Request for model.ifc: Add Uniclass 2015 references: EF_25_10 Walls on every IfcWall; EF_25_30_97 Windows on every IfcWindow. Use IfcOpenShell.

First a look at what the model holds.

```python
import ifcopenshell

model = ifcopenshell.open("model.ifc")
print(model.schema)
print("classifications:", [c.Name for c in model.by_type("IfcClassification")])
for ifc_class in ("IfcDoor", "IfcRoof", "IfcStair", "IfcWall", "IfcWindow"):
    print(ifc_class, len(model.by_type(ifc_class)))
```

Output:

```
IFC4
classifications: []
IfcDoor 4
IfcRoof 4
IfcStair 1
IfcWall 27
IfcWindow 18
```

```python
import ifcopenshell
import ifcopenshell.api.classification

model = ifcopenshell.open("model.ifc")

system = ifcopenshell.api.classification.add_classification(model, classification="Uniclass 2015")

codes = {
    "IfcWall": ("EF_25_10", "Walls"),
    "IfcWindow": ("EF_25_30_97", "Windows"),
}
for ifc_class, (code, name) in codes.items():
    products = model.by_type(ifc_class)
    ifcopenshell.api.classification.add_reference(
        model, products=products, classification=system, identification=code, name=name
    )
    print(code, len(products))

model.write("model_v2.ifc")
```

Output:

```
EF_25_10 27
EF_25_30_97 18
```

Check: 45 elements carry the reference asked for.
